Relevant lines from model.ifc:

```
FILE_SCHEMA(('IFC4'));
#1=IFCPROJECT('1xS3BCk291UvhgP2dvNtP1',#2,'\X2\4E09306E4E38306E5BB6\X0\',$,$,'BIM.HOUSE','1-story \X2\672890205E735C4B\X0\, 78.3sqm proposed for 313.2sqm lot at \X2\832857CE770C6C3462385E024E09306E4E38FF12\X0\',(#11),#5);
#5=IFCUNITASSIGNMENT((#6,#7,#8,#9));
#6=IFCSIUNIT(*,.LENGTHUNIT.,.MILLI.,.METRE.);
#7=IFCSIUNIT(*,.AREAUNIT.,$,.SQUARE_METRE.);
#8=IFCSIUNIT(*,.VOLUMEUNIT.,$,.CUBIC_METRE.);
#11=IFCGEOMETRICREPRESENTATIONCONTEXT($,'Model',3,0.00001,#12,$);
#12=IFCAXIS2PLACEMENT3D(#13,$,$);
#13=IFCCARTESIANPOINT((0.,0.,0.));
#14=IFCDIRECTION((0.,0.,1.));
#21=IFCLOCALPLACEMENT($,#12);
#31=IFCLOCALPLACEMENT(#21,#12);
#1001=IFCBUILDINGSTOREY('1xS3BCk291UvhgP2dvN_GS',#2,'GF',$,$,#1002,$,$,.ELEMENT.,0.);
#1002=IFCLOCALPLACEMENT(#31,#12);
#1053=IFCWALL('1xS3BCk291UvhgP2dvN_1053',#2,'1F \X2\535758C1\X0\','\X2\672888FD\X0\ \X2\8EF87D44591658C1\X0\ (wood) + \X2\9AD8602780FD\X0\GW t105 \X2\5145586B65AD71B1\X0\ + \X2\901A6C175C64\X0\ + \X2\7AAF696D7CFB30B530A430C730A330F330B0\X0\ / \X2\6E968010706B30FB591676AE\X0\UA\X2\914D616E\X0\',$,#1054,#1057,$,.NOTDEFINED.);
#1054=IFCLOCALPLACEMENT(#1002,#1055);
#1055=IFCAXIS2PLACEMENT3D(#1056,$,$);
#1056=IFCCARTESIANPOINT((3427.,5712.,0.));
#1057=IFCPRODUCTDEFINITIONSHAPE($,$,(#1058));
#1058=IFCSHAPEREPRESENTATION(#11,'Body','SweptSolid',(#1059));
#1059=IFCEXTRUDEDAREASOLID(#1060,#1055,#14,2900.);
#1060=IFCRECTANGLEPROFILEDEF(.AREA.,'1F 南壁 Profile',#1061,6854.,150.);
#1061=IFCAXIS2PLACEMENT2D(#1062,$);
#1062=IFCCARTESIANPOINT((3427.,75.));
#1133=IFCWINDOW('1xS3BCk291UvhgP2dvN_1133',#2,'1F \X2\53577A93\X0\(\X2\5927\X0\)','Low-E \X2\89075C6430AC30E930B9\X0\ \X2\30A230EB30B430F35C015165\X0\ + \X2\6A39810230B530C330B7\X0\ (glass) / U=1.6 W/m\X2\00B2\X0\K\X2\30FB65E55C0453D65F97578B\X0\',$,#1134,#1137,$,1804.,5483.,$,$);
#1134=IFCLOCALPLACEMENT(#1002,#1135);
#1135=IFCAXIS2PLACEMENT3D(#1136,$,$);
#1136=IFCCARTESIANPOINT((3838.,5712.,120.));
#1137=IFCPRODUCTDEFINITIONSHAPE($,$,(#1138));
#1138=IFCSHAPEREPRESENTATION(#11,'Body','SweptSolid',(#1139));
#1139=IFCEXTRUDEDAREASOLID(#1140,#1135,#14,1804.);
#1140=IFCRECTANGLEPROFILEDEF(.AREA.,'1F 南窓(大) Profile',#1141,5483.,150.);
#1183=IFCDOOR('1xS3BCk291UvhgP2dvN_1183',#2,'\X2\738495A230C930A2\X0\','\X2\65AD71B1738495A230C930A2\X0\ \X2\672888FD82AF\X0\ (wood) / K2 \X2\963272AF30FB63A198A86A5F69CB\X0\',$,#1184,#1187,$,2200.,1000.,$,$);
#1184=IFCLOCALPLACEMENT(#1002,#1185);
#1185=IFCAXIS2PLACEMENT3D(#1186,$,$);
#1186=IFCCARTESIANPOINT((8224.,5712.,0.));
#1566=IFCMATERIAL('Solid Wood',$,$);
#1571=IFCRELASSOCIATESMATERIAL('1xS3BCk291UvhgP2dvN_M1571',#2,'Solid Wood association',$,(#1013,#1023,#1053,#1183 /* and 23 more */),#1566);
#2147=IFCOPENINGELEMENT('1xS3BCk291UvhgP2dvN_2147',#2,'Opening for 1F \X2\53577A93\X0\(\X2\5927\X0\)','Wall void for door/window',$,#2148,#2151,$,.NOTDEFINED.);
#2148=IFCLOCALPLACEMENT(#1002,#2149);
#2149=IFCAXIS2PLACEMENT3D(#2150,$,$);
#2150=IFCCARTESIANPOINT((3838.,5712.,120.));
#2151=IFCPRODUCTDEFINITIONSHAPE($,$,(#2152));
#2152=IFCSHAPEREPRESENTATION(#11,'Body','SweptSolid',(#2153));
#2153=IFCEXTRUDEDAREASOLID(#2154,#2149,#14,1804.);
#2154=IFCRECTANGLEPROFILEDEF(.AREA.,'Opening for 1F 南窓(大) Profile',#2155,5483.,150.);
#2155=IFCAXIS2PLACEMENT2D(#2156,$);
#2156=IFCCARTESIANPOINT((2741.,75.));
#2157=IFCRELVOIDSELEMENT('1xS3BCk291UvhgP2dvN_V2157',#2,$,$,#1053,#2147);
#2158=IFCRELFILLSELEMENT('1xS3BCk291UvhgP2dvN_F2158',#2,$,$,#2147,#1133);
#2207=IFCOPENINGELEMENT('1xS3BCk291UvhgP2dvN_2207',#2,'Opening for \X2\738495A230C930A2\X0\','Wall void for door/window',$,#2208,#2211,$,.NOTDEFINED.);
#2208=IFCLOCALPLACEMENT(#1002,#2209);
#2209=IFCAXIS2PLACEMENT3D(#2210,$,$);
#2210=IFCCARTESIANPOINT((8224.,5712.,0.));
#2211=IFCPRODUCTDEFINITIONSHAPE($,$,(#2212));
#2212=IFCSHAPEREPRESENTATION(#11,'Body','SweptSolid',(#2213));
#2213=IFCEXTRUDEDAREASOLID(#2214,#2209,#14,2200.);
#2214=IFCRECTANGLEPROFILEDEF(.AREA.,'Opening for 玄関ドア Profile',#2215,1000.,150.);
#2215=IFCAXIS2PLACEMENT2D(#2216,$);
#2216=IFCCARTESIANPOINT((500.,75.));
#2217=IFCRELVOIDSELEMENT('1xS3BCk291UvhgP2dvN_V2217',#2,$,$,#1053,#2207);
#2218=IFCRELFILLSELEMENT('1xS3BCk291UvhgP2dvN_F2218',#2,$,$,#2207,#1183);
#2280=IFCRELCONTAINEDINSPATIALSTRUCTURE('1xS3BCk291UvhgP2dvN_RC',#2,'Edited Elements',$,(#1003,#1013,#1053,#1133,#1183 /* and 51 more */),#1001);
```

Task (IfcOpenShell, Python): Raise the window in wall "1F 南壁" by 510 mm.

```python
import numpy as np
import ifcopenshell
import ifcopenshell.api.geometry
import ifcopenshell.util.placement
import ifcopenshell.util.unit

model = ifcopenshell.open("model.ifc")
unit_scale = ifcopenshell.util.unit.calculate_unit_scale(model)

window = model.by_guid("1xS3BCk291UvhgP2dvN_1133")
opening = window.FillsVoids[0].RelatingOpeningElement
dz = 0.51 / unit_scale

shift = np.array([0.0, 0.0, dz])
# The window is not placed relative to its opening, so move both.
for product in (opening, window):
    matrix = ifcopenshell.util.placement.get_local_placement(product.ObjectPlacement)
    matrix[:3, 3] += shift
    ifcopenshell.api.geometry.edit_object_placement(model, product=product, matrix=matrix, is_si=False)

print(f"moved by {dz * unit_scale:+.3f} m")

model.write("model_v2.ifc")
```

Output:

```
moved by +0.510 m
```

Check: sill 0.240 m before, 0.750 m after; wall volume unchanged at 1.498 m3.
